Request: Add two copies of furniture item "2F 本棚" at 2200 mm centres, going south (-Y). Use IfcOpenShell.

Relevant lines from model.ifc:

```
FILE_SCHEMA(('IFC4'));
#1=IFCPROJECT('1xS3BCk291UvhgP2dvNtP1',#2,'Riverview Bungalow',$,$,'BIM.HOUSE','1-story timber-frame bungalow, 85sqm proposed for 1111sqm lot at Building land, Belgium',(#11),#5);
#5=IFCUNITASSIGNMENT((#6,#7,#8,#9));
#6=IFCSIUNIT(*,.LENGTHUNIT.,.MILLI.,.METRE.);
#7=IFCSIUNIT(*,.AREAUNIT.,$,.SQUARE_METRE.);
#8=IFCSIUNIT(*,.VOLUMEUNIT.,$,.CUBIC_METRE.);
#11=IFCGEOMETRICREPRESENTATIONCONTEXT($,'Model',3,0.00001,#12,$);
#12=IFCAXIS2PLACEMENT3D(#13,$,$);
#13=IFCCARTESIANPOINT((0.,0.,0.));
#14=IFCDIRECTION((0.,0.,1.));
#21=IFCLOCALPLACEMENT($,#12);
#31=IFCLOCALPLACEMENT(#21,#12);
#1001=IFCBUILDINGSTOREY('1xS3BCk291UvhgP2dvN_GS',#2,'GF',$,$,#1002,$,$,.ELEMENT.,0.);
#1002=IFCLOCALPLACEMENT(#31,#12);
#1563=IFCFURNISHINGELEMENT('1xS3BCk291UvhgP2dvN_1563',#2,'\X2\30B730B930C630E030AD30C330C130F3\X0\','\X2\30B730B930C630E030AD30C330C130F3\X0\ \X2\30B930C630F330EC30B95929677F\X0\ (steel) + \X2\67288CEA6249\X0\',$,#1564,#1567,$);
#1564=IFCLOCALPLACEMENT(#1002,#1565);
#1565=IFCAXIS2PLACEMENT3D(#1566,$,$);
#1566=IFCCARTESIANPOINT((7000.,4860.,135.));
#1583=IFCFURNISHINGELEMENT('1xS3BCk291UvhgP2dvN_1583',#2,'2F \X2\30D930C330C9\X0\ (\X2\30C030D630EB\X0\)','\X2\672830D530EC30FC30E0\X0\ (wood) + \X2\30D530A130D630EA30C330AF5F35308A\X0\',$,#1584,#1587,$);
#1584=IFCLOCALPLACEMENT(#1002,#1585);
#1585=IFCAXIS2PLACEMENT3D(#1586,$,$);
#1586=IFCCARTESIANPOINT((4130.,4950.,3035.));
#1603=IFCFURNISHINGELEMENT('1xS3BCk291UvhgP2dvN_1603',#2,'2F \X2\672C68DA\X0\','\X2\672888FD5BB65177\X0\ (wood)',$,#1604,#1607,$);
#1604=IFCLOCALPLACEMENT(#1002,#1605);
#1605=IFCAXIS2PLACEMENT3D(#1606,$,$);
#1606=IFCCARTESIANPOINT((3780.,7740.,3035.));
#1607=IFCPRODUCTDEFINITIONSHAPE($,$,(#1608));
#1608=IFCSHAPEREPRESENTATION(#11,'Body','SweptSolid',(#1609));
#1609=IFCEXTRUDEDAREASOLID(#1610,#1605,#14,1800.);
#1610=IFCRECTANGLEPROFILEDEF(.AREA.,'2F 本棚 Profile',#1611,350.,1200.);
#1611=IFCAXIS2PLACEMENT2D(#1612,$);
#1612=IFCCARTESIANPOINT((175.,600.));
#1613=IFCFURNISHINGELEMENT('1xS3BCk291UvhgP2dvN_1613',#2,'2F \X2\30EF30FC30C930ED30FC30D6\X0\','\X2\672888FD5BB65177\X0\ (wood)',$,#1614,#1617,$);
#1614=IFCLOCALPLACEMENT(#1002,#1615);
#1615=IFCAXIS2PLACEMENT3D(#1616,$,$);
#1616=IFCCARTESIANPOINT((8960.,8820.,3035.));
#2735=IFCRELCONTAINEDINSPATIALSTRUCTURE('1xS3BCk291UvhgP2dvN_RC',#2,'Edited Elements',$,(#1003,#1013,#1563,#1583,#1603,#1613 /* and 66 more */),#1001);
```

```python
import numpy as np
import ifcopenshell
import ifcopenshell.api.geometry
import ifcopenshell.api.root
import ifcopenshell.util.element
import ifcopenshell.util.placement
import ifcopenshell.util.unit

model = ifcopenshell.open("model.ifc")
unit_scale = ifcopenshell.util.unit.calculate_unit_scale(model)


def reuse_history(source, copy):
    """copy_class also copies each property set's owner history, people and application; keep the originals."""
    for rel in copy.IsDefinedBy:
        if rel.is_a("IfcRelDefinesByProperties") and (history := rel.RelatingPropertyDefinition.OwnerHistory):
            rel.RelatingPropertyDefinition.OwnerHistory = source.OwnerHistory
            ifcopenshell.util.element.remove_deep2(model, history)


source = model.by_id(1603)
base = ifcopenshell.util.placement.get_local_placement(source.ObjectPlacement)
step = np.array([0.0, -1.0, 0.0]) * 2.2 / unit_scale

for i in range(1, 3):
    copy = ifcopenshell.api.root.copy_class(model, product=source)
    copy.Representation = ifcopenshell.util.element.copy_deep(
        model, source.Representation, exclude=["IfcGeometricRepresentationContext", "IfcRepresentationMap"]
    )
    reuse_history(source, copy)
    matrix = base.copy()
    matrix[:3, 3] += i * step
    print("added at", matrix[:3, 3].round(3) + 0.0)
    ifcopenshell.api.geometry.edit_object_placement(model, product=copy, matrix=matrix, is_si=False)

model.write("model-out.ifc")
```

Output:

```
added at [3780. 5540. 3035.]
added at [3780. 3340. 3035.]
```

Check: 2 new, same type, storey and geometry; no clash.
